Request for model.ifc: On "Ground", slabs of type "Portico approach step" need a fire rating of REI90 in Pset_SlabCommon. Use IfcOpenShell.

First a look at what the model holds.

```python
import ifcopenshell
import ifcopenshell.util.element

model = ifcopenshell.open("model.ifc")
print(model.schema)
storey = next(s for s in model.by_type("IfcBuildingStorey") if s.Name == "Ground")
slabs = [e for e in ifcopenshell.util.element.get_decomposition(storey) if e.is_a("IfcSlab")]
seen = {}
for e in slabs:
    element_type = ifcopenshell.util.element.get_type(e)
    key = (element_type.Name if element_type != e and element_type else None, ifcopenshell.util.element.get_pset(e, "Pset_SlabCommon", "FireRating"))
    seen[key] = seen.get(key, 0) + 1
for (name, value), count in sorted(seen.items(), key=str):
    print(count, "x", name, "|", value)
```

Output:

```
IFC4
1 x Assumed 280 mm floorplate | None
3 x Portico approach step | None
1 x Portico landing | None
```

```python
import ifcopenshell
import ifcopenshell.api.pset
import ifcopenshell.util.element

model = ifcopenshell.open("model.ifc")

storey = next(s for s in model.by_type("IfcBuildingStorey") if s.Name == "Ground")
slabs = [e for e in ifcopenshell.util.element.get_decomposition(storey) if e.is_a("IfcSlab")]

count = 0
for e in slabs:
    element_type = ifcopenshell.util.element.get_type(e)
    if element_type in (None, e) or element_type.Name != "Portico approach step":
        continue
    # add_pset returns the element's existing set when there is one.
    pset = ifcopenshell.api.pset.add_pset(model, product=e, name="Pset_SlabCommon")
    ifcopenshell.api.pset.edit_pset(model, pset=pset, properties={"FireRating": "REI90"})
    count += 1

print(count, "slabs updated")

model.write("model_edited.ifc")
```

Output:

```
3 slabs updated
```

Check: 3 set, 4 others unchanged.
